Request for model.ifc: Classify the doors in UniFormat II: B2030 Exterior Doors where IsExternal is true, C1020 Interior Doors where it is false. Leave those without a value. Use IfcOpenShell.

First a look at what the model holds.

```python
import ifcopenshell
import ifcopenshell.util.element

model = ifcopenshell.open("model.ifc")
print(model.schema)
print("classifications:", [c.Name for c in model.by_type("IfcClassification")])
values = [ifcopenshell.util.element.get_pset(e, "Pset_DoorCommon", "IsExternal") for e in model.by_type("IfcDoor")]
for value in (True, False, None):
    print("IsExternal", value, values.count(value))
```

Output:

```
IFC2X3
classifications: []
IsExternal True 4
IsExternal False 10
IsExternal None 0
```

```python
import ifcopenshell
import ifcopenshell.api.classification
import ifcopenshell.util.element

model = ifcopenshell.open("model.ifc")

# IFC2X3 requires Source and Edition and has no link from the project to the system.
system = model.create_entity("IfcClassification", Source="ASTM", Edition="E1557", Name="UniFormat II")

doors = model.by_type("IfcDoor")
external = {e: ifcopenshell.util.element.get_pset(e, "Pset_DoorCommon", "IsExternal") for e in doors}
for flag, code, name in ((True, "B2030", "Exterior Doors"), (False, "C1020", "Interior Doors")):
    products = [e for e in doors if external[e] is flag]
    ifcopenshell.api.classification.add_reference(
        model, products=products, classification=system, identification=code, name=name
    )
    print(code, len(products))

model.write("model-out.ifc")
```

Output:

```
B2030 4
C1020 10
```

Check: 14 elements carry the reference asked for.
